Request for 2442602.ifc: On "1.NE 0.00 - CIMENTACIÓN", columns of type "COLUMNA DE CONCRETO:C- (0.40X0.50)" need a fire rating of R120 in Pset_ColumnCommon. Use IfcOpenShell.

First a look at what the model holds.

```python
import ifcopenshell
import ifcopenshell.util.element

model = ifcopenshell.open("2442602.ifc")
print(model.schema)
storey = next(s for s in model.by_type("IfcBuildingStorey") if s.Name == "1.NE 0.00 - CIMENTACIÓN")
columns = [e for e in ifcopenshell.util.element.get_decomposition(storey) if e.is_a("IfcColumn")]
seen = {}
for e in columns:
    element_type = ifcopenshell.util.element.get_type(e)
    key = (element_type.Name if element_type != e and element_type else None, ifcopenshell.util.element.get_pset(e, "Pset_ColumnCommon", "FireRating"))
    seen[key] = seen.get(key, 0) + 1
for (name, value), count in sorted(seen.items(), key=str):
    print(count, "x", name, "|", value)
```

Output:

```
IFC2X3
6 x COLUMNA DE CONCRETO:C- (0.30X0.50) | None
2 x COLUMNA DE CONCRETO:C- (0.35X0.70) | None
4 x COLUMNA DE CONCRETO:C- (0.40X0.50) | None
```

```python
import ifcopenshell
import ifcopenshell.api.pset
import ifcopenshell.util.element

model = ifcopenshell.open("2442602.ifc")

storey = next(s for s in model.by_type("IfcBuildingStorey") if s.Name == "1.NE 0.00 - CIMENTACIÓN")
columns = [e for e in ifcopenshell.util.element.get_decomposition(storey) if e.is_a("IfcColumn")]

count = 0
for e in columns:
    element_type = ifcopenshell.util.element.get_type(e)
    if element_type in (None, e) or element_type.Name != "COLUMNA DE CONCRETO:C- (0.40X0.50)":
        continue
    # add_pset returns the element's existing set when there is one.
    pset = ifcopenshell.api.pset.add_pset(model, product=e, name="Pset_ColumnCommon")
    ifcopenshell.api.pset.edit_pset(model, pset=pset, properties={"FireRating": "R120"})
    count += 1

print(count, "columns updated")

model.write("2442602_rev.ifc")
```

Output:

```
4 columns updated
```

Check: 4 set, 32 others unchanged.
